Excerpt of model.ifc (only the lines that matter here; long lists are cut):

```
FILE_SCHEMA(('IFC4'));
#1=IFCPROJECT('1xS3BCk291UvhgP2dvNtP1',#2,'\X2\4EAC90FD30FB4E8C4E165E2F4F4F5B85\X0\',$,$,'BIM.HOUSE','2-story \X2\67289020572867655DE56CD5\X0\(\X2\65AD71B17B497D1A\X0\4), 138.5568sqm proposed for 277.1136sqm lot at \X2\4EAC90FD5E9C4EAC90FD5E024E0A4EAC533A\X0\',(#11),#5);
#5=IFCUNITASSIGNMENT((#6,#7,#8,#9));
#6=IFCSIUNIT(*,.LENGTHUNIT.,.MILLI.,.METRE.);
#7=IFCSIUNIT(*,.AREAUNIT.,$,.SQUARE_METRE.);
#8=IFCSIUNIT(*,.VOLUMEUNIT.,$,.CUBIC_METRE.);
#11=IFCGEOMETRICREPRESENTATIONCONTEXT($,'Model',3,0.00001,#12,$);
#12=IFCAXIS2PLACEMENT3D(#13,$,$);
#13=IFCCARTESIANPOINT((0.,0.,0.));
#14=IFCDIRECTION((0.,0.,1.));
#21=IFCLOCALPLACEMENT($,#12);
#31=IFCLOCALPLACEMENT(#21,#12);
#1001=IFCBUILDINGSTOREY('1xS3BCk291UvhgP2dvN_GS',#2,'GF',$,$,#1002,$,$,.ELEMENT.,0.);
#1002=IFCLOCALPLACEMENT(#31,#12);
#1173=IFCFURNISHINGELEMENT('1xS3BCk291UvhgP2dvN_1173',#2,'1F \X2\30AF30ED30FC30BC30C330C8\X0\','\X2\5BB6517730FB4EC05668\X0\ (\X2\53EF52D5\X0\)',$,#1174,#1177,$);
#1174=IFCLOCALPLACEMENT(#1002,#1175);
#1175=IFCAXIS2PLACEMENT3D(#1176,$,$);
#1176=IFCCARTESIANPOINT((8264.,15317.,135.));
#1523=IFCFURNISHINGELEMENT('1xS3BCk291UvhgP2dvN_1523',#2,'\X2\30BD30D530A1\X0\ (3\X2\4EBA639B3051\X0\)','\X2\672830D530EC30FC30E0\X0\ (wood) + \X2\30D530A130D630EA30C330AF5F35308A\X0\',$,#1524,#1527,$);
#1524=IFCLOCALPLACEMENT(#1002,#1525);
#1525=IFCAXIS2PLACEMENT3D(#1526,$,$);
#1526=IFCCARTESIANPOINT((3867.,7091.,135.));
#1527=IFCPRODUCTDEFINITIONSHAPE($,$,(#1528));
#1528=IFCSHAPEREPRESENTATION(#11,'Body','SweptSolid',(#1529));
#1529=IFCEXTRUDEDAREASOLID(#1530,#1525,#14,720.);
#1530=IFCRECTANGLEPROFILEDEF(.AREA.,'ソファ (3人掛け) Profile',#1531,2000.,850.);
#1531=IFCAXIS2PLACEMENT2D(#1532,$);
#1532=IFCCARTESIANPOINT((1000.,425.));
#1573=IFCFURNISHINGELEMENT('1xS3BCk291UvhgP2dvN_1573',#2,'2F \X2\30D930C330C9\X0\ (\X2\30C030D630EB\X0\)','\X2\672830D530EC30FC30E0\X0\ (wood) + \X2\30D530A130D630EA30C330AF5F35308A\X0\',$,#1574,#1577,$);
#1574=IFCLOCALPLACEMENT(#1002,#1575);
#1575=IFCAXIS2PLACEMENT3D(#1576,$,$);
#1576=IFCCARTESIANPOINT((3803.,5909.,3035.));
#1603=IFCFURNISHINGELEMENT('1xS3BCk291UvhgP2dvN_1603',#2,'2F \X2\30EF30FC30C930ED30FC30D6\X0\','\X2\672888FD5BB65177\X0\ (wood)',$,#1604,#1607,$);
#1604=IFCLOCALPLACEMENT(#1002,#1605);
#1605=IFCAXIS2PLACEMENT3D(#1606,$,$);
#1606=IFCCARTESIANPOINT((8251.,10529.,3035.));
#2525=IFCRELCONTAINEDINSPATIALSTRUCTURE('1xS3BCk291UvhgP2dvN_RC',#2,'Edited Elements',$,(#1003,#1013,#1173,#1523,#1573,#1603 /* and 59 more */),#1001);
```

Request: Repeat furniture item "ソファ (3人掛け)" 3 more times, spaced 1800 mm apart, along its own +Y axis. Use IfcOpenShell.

```python
import ifcopenshell
import ifcopenshell.api.geometry
import ifcopenshell.api.root
import ifcopenshell.util.element
import ifcopenshell.util.placement

model = ifcopenshell.open("model.ifc")


def reuse_history(source, copy):
    """copy_class also copies each property set's owner history, people and application; keep the originals."""
    for rel in copy.IsDefinedBy:
        if rel.is_a("IfcRelDefinesByProperties") and (history := rel.RelatingPropertyDefinition.OwnerHistory):
            rel.RelatingPropertyDefinition.OwnerHistory = source.OwnerHistory
            ifcopenshell.util.element.remove_deep2(model, history)


source = model.by_guid("1xS3BCk291UvhgP2dvN_1523")
base = ifcopenshell.util.placement.get_local_placement(source.ObjectPlacement)
step = base[:3, 1] * 1800.0

for i in range(1, 4):
    copy = ifcopenshell.api.root.copy_class(model, product=source)
    copy.Representation = ifcopenshell.util.element.copy_deep(
        model, source.Representation, exclude=["IfcGeometricRepresentationContext", "IfcRepresentationMap"]
    )
    reuse_history(source, copy)
    matrix = base.copy()
    matrix[:3, 3] += i * step
    print("added at", matrix[:3, 3].round(3) + 0.0)
    ifcopenshell.api.geometry.edit_object_placement(model, product=copy, matrix=matrix, is_si=False)

model.write("model_edited.ifc")
```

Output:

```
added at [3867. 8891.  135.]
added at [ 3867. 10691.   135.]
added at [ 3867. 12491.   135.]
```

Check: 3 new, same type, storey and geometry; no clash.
